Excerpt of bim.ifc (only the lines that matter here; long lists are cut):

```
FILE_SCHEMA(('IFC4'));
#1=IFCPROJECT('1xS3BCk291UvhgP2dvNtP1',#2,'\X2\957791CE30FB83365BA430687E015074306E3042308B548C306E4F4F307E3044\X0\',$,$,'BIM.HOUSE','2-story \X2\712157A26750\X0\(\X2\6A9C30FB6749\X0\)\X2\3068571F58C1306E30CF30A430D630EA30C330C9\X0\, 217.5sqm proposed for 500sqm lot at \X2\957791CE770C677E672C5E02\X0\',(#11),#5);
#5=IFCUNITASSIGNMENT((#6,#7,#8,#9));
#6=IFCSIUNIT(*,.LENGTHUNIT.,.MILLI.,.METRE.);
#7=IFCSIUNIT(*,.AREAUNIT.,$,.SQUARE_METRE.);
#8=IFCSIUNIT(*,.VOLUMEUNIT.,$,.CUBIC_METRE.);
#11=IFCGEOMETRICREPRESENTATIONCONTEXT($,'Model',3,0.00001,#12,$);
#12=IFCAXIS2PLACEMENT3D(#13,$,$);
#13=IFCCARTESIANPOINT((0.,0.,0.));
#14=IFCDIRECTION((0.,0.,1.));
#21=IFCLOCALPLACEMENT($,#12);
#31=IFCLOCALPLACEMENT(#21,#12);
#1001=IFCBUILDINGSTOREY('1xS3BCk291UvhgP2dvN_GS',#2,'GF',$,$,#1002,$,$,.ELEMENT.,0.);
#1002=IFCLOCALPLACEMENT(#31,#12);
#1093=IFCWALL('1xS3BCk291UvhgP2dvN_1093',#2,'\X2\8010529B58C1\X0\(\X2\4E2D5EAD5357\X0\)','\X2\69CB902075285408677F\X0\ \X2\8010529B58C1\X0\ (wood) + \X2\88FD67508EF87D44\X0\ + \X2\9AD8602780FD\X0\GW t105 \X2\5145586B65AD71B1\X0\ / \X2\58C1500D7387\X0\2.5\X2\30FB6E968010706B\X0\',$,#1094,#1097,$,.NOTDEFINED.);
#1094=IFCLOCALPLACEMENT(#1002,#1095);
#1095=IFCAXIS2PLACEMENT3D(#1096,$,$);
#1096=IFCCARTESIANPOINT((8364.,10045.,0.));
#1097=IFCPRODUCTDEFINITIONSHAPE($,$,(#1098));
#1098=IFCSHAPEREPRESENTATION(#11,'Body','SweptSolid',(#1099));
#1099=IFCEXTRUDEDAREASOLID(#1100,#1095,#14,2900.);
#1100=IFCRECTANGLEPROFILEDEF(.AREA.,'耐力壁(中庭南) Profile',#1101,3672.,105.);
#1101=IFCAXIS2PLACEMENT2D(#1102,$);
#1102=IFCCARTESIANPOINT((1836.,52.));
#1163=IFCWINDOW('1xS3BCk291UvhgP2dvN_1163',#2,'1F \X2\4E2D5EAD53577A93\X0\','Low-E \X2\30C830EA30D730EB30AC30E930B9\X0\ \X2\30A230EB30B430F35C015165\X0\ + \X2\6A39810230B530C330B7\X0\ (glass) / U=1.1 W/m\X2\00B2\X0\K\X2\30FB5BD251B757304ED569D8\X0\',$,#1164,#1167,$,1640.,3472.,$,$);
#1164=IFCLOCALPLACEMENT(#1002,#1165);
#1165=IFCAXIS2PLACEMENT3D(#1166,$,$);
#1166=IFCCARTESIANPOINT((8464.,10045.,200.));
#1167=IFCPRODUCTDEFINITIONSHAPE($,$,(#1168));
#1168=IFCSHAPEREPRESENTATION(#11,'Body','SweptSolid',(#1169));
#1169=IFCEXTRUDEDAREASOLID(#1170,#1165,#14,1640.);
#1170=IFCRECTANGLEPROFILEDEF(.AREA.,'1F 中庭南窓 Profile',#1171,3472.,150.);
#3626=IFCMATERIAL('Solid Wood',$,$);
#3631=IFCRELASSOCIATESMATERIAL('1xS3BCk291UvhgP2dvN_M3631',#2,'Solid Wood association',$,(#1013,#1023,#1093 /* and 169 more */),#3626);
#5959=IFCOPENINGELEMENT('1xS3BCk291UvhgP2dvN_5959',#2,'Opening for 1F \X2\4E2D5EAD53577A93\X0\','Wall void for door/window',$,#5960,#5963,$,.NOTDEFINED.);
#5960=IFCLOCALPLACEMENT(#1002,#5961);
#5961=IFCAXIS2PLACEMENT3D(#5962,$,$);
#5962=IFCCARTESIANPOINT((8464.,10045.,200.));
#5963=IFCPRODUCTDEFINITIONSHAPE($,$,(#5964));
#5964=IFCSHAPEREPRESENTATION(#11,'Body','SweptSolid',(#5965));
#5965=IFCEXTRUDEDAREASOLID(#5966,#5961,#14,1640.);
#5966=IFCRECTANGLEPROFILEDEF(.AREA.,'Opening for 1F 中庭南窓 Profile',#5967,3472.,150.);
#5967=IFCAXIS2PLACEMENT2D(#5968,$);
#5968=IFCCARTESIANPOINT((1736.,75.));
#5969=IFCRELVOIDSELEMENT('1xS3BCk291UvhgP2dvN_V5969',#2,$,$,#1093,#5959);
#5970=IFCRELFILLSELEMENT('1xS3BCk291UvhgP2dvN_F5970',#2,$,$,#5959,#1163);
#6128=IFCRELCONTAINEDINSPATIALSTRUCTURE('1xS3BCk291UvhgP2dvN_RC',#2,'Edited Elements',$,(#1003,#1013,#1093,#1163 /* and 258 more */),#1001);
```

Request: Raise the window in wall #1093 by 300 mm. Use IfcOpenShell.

```python
import numpy as np
import ifcopenshell
import ifcopenshell.api.geometry
import ifcopenshell.util.placement
import ifcopenshell.util.unit

model = ifcopenshell.open("bim.ifc")
unit_scale = ifcopenshell.util.unit.calculate_unit_scale(model)

window = model.by_guid("1xS3BCk291UvhgP2dvN_1163")
opening = window.FillsVoids[0].RelatingOpeningElement
dz = 300.0

shift = np.array([0.0, 0.0, dz])
# The window is not placed relative to its opening, so move both.
for product in (opening, window):
    matrix = ifcopenshell.util.placement.get_local_placement(product.ObjectPlacement)
    matrix[:3, 3] += shift
    ifcopenshell.api.geometry.edit_object_placement(model, product=product, matrix=matrix, is_si=False)

print(f"moved by {dz * unit_scale:+.3f} m")

model.write("bim_v2.ifc")
```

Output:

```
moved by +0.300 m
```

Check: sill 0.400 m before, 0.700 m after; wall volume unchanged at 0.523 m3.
